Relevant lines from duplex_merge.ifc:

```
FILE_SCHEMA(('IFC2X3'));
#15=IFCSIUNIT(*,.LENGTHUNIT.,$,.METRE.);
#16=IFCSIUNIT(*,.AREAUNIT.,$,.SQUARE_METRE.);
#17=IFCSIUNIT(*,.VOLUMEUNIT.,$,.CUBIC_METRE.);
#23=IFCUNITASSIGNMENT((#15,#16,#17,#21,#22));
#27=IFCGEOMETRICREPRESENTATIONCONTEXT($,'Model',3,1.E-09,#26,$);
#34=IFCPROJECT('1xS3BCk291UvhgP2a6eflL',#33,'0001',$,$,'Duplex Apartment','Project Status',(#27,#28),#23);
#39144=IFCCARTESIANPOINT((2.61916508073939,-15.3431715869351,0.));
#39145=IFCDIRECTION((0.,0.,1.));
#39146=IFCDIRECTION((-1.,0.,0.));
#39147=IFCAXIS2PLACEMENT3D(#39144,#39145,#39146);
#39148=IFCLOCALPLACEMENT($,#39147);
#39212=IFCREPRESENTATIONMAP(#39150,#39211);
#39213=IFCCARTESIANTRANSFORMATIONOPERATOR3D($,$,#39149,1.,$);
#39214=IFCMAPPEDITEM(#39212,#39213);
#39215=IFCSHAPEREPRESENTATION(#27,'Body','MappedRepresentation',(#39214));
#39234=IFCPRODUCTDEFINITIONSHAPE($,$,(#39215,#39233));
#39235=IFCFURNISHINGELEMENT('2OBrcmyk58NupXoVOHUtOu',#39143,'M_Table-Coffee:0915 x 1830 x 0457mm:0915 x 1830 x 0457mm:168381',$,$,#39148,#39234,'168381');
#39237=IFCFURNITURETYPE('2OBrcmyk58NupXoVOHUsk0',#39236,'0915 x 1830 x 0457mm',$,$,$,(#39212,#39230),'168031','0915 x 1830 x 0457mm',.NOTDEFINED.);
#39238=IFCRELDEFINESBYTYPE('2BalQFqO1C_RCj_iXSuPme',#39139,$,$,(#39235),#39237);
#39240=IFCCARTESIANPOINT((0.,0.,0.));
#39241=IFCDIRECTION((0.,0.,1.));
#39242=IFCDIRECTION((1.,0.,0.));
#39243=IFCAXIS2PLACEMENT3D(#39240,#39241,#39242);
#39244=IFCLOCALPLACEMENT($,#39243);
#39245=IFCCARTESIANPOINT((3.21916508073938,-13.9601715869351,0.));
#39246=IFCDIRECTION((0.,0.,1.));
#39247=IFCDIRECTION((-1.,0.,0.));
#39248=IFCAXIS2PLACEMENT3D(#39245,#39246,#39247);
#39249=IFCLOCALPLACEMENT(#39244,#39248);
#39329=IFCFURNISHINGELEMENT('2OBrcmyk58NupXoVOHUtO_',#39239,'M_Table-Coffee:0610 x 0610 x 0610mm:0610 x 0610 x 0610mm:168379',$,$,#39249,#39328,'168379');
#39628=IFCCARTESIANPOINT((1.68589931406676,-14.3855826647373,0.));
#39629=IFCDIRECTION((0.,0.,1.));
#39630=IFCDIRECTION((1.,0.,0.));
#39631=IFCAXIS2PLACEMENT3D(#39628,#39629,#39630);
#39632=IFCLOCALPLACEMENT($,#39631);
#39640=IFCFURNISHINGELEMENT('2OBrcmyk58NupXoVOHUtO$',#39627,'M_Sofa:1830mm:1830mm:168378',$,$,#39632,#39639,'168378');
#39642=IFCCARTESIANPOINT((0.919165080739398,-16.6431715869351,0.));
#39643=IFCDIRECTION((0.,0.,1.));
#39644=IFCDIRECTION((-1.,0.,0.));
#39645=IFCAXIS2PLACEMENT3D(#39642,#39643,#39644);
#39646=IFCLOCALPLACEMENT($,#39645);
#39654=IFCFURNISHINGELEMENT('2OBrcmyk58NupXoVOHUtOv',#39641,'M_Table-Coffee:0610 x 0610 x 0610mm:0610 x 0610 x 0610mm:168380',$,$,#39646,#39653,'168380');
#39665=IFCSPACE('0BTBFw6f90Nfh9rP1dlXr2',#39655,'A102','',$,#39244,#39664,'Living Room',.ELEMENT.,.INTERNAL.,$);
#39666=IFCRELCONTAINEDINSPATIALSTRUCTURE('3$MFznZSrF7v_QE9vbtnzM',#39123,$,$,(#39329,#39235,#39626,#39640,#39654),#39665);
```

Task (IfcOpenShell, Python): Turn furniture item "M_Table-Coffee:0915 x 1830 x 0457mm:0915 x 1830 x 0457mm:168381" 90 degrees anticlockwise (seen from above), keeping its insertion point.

```python
import ifcopenshell
import ifcopenshell.api.geometry
import ifcopenshell.util.placement

model = ifcopenshell.open("duplex_merge.ifc")

item = model.by_guid("2OBrcmyk58NupXoVOHUtOu")
matrix = ifcopenshell.util.placement.get_local_placement(item.ObjectPlacement)
matrix = matrix @ ifcopenshell.util.placement.rotation(90, "Z")
ifcopenshell.api.geometry.edit_object_placement(model, product=item, matrix=matrix, is_si=False)

print(ifcopenshell.util.placement.get_local_placement(item.ObjectPlacement).round(3) + 0.0)

model.write("duplex_merge_v2.ifc")
```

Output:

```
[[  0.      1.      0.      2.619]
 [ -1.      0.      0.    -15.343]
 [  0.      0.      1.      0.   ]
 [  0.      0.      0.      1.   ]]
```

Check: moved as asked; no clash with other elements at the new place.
